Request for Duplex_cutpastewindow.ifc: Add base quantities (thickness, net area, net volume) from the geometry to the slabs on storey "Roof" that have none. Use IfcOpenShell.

First a look at what the model holds.

```python
import ifcopenshell
import ifcopenshell.util.element
import ifcopenshell.util.unit

model = ifcopenshell.open("Duplex_cutpastewindow.ifc")
print(model.schema)
for unit_type in ("LENGTHUNIT", "AREAUNIT", "VOLUMEUNIT"):
    print(unit_type, ifcopenshell.util.unit.calculate_unit_scale(model, unit_type))
storey = next(s for s in model.by_type("IfcBuildingStorey") if s.Name == "Roof")
slabs = [e for e in ifcopenshell.util.element.get_decomposition(storey) if e.is_a("IfcSlab")]
for e in sorted(slabs, key=lambda e: e.id()):
    print(e.id(), e.is_a(), e.Name, list(ifcopenshell.util.element.get_psets(e, qtos_only=True)), sep=" | ")
```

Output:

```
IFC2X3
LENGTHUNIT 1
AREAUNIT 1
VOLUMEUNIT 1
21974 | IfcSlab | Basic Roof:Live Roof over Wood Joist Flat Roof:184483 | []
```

```python
import ifcopenshell
import ifcopenshell.api.pset
import ifcopenshell.geom
import ifcopenshell.util.element
import ifcopenshell.util.shape
import ifcopenshell.util.unit

model = ifcopenshell.open("Duplex_cutpastewindow.ifc")
unit_scale = ifcopenshell.util.unit.calculate_unit_scale(model)
area_scale = ifcopenshell.util.unit.calculate_unit_scale(model, "AREAUNIT")
volume_scale = ifcopenshell.util.unit.calculate_unit_scale(model, "VOLUMEUNIT")
settings = ifcopenshell.geom.settings()

storey = next(s for s in model.by_type("IfcBuildingStorey") if s.Name == "Roof")
slabs = [e for e in ifcopenshell.util.element.get_decomposition(storey) if e.is_a("IfcSlab")]

for e in sorted(slabs, key=lambda e: e.id()):
    if ifcopenshell.util.element.get_psets(e, qtos_only=True, should_inherit=False):
        continue
    # Geometry comes back in metres, in the element's own axes.
    shape = ifcopenshell.geom.create_shape(settings, e)
    values = {
        "Width": ifcopenshell.util.shape.get_z(shape.geometry) / unit_scale,
        "NetArea": ifcopenshell.util.shape.get_footprint_area(shape.geometry) / area_scale,
        "NetVolume": ifcopenshell.util.shape.get_volume(shape.geometry) / volume_scale,
    }
    qto = ifcopenshell.api.pset.add_qto(model, product=e, name="BaseQuantities")
    ifcopenshell.api.pset.edit_qto(model, qto=qto, properties=values)
    print(e.id(), {k: round(v, 3) for k, v in values.items()})

model.write("Duplex_cutpastewindow_updated.ifc")
```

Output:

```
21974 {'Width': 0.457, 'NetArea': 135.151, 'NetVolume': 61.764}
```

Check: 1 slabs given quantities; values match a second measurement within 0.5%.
